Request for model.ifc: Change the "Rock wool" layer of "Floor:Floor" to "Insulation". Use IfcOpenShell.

First a look at what the model holds.

```python
import ifcopenshell
import ifcopenshell.util.element

model = ifcopenshell.open("model.ifc")
print(model.schema)
for layer_set in model.by_type("IfcMaterialLayerSet"):
    if layer_set.LayerSetName == "Floor:Floor":
        for layer in layer_set.MaterialLayers:
            print(layer.id(), layer.Material and layer.Material.Name, layer.LayerThickness, sep=" | ")
        print(len(ifcopenshell.util.element.get_elements_by_material(model, layer_set)), "elements and types use it")
print(sorted(m.Name for m in model.by_type("IfcMaterial") if m.Name)[:60])
```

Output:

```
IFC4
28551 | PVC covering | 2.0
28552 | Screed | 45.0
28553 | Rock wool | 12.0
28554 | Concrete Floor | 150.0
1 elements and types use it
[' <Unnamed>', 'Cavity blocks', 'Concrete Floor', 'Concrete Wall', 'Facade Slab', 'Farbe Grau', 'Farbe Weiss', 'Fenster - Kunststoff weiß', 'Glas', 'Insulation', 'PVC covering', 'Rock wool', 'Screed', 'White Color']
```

```python
import ifcopenshell
import ifcopenshell.api.material

model = ifcopenshell.open("model.ifc")

layer_set = next(s for s in model.by_type("IfcMaterialLayerSet") if s.LayerSetName == "Floor:Floor")
layer = next(l for l in layer_set.MaterialLayers if l.Material and l.Material.Name == "Rock wool")
material = next(m for m in model.by_type("IfcMaterial") if m.Name == "Insulation")

# Point this one layer at the other material; renaming the old one would change it everywhere.
ifcopenshell.api.material.edit_layer(model, layer=layer, attributes={}, material=material)

print([l.Material.Name if l.Material else None for l in layer_set.MaterialLayers])

model.write("model_v2.ifc")
```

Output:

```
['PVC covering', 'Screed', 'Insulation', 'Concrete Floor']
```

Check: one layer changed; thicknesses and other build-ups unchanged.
